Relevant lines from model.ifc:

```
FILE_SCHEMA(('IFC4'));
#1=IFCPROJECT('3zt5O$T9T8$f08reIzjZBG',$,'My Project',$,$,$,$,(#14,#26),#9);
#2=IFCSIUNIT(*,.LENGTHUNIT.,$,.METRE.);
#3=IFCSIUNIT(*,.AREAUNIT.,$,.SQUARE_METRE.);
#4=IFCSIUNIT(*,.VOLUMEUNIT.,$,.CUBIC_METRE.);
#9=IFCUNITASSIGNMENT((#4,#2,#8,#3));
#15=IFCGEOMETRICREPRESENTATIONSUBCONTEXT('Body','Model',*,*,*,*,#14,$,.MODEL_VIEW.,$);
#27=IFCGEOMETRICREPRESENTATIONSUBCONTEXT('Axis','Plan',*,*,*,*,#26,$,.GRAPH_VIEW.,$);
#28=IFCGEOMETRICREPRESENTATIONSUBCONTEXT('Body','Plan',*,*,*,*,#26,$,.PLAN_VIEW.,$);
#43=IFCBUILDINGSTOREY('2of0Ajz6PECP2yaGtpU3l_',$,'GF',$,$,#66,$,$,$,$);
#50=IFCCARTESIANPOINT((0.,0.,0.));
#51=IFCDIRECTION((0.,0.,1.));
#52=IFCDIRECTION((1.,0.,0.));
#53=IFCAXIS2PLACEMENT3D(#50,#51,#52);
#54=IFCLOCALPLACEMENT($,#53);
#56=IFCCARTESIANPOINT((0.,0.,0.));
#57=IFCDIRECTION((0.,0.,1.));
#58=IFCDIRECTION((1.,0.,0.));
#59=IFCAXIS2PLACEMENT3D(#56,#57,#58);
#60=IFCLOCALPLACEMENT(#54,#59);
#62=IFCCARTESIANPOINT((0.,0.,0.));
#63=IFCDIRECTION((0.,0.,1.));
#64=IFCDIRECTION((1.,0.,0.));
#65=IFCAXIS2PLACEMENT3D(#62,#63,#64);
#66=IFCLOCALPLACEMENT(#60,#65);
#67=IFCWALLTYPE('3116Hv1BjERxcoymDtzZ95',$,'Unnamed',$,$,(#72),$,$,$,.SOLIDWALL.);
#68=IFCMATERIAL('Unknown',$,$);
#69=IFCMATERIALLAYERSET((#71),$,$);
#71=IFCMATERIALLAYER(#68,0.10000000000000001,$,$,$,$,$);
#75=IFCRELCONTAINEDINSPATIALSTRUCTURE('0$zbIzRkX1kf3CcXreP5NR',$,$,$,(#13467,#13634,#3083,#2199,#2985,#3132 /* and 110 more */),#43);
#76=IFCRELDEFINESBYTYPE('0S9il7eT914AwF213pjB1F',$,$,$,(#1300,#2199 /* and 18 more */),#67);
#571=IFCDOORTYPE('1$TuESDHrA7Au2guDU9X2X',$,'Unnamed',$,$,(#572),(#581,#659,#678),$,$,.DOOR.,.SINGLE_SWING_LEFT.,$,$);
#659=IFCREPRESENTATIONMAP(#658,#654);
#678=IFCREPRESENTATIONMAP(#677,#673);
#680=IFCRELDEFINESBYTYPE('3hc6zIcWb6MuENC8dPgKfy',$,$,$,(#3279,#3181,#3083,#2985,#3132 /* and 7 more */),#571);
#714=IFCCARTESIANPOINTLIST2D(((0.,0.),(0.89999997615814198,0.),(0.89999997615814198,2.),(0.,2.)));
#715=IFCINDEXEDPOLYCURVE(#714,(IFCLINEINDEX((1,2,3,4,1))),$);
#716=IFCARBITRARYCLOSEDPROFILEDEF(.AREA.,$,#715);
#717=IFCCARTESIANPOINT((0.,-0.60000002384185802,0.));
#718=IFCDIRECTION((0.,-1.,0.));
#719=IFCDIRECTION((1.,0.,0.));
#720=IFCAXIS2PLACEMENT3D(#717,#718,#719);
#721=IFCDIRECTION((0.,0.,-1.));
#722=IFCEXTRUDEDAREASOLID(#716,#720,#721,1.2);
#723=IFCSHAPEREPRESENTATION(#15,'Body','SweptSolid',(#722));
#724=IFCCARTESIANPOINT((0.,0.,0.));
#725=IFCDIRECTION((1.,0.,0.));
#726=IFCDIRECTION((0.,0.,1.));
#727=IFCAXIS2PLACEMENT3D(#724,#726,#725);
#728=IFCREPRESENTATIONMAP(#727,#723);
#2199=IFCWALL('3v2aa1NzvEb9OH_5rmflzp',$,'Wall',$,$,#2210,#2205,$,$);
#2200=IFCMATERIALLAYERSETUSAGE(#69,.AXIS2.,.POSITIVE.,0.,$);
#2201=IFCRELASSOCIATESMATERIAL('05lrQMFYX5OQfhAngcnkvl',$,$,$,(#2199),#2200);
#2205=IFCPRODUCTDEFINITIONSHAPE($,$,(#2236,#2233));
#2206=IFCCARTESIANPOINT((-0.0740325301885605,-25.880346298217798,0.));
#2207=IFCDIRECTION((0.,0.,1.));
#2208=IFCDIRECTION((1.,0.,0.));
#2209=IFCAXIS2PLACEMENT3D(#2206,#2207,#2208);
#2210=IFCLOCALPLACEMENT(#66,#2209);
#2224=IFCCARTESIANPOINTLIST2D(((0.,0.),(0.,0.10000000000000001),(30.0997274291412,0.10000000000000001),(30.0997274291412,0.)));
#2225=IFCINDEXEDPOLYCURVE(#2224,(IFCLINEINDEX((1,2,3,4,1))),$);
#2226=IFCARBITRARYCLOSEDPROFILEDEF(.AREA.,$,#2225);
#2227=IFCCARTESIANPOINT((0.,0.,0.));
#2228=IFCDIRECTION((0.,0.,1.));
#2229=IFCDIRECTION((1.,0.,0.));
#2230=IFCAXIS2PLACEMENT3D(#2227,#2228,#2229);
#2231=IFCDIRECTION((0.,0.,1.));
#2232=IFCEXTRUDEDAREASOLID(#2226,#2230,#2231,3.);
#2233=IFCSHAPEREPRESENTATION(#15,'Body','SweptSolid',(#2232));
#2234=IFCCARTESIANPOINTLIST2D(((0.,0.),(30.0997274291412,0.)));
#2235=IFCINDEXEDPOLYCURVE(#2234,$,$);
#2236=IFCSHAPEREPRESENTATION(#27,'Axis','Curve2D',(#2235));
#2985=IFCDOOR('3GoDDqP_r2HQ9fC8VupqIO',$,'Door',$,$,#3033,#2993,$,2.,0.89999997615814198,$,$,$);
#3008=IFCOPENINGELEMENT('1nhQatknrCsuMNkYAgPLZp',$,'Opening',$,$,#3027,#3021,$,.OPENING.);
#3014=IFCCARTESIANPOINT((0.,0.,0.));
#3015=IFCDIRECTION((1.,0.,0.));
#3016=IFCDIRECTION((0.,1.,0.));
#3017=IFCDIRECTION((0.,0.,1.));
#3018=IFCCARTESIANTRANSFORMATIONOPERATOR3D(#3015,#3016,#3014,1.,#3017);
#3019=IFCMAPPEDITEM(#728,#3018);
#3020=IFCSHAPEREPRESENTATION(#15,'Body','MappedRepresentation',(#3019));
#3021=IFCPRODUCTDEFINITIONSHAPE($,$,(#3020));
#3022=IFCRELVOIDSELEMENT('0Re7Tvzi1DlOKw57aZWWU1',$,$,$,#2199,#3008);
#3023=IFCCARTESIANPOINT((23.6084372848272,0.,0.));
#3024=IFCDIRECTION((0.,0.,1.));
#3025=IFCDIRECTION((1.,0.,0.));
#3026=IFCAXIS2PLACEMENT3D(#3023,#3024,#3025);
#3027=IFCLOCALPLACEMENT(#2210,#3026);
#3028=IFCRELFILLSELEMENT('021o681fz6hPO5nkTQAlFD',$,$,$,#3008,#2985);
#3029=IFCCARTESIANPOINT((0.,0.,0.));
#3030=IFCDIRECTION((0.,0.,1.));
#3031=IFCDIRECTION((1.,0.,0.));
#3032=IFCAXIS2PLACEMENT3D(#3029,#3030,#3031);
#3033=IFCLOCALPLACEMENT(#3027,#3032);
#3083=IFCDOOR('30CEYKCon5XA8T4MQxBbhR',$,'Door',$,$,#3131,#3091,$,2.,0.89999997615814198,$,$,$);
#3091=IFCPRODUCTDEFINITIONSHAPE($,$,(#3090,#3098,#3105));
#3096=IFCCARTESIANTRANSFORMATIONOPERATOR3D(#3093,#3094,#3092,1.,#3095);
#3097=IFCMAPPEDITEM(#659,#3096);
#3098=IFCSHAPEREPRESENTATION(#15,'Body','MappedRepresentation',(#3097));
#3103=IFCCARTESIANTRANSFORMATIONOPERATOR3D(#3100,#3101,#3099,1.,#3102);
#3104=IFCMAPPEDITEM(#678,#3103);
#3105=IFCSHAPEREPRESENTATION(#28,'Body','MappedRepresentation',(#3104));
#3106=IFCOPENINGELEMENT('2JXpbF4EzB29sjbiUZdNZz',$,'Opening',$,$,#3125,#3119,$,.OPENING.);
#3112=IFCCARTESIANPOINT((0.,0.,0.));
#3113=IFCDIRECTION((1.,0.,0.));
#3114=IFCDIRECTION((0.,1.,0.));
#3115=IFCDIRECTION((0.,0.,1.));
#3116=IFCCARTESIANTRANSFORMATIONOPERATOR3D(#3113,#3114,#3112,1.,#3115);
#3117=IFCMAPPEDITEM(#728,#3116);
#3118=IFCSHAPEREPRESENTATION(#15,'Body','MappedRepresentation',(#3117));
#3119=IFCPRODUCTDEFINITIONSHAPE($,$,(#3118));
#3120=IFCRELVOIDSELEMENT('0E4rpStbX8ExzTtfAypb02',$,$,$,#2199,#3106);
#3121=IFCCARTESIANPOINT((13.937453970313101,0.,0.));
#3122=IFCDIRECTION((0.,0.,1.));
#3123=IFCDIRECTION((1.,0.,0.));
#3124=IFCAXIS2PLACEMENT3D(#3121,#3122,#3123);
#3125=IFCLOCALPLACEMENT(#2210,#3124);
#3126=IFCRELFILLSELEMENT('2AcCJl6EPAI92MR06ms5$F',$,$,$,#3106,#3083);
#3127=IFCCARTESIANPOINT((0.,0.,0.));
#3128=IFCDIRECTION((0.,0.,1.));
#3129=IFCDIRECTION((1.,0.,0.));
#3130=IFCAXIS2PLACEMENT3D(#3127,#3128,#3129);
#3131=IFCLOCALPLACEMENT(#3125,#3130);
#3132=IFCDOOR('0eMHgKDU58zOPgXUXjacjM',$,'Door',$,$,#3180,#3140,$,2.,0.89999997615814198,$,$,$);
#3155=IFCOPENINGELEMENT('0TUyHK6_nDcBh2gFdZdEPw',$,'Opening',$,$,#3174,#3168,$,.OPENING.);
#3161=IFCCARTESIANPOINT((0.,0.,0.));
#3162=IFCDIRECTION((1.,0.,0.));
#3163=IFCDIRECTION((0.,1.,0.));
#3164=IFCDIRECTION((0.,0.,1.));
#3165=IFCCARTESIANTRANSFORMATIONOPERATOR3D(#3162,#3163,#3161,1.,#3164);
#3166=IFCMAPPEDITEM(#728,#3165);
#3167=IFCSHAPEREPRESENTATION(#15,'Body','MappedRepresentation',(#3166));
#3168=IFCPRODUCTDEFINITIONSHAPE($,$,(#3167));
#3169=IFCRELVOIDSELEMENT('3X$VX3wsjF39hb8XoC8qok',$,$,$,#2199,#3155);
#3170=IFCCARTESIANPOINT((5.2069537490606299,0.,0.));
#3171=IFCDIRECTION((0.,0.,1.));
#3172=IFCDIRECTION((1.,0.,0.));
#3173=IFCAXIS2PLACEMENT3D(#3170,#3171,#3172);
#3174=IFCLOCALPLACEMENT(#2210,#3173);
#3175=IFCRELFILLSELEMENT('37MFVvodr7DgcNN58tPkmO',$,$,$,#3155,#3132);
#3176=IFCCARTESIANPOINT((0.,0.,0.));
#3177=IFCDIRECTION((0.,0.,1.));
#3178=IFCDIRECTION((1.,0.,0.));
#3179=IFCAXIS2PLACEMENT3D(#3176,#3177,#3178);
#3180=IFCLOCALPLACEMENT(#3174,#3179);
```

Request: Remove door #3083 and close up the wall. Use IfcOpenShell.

```python
import ifcopenshell
import ifcopenshell.api.feature
import ifcopenshell.api.root
import ifcopenshell.geom
import ifcopenshell.util.shape

model = ifcopenshell.open("model.ifc")
settings = ifcopenshell.geom.settings()


def volume(element):
    """Net volume in cubic metres, openings subtracted."""
    shape = ifcopenshell.geom.create_shape(settings, element)
    return ifcopenshell.util.shape.get_volume(shape.geometry)


door = model.by_guid("30CEYKCon5XA8T4MQxBbhR")
opening = door.FillsVoids[0].RelatingOpeningElement
wall = opening.VoidsElements[0].RelatingBuildingElement
before = volume(wall)

ifcopenshell.api.root.remove_product(model, product=door)
ifcopenshell.api.feature.remove_feature(model, feature=opening)

after = volume(wall)

print(f"wall volume {before:.3f} -> {after:.3f} m3")

model.write("model-out.ifc")
```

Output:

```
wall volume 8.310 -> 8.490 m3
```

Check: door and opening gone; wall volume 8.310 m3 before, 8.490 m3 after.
